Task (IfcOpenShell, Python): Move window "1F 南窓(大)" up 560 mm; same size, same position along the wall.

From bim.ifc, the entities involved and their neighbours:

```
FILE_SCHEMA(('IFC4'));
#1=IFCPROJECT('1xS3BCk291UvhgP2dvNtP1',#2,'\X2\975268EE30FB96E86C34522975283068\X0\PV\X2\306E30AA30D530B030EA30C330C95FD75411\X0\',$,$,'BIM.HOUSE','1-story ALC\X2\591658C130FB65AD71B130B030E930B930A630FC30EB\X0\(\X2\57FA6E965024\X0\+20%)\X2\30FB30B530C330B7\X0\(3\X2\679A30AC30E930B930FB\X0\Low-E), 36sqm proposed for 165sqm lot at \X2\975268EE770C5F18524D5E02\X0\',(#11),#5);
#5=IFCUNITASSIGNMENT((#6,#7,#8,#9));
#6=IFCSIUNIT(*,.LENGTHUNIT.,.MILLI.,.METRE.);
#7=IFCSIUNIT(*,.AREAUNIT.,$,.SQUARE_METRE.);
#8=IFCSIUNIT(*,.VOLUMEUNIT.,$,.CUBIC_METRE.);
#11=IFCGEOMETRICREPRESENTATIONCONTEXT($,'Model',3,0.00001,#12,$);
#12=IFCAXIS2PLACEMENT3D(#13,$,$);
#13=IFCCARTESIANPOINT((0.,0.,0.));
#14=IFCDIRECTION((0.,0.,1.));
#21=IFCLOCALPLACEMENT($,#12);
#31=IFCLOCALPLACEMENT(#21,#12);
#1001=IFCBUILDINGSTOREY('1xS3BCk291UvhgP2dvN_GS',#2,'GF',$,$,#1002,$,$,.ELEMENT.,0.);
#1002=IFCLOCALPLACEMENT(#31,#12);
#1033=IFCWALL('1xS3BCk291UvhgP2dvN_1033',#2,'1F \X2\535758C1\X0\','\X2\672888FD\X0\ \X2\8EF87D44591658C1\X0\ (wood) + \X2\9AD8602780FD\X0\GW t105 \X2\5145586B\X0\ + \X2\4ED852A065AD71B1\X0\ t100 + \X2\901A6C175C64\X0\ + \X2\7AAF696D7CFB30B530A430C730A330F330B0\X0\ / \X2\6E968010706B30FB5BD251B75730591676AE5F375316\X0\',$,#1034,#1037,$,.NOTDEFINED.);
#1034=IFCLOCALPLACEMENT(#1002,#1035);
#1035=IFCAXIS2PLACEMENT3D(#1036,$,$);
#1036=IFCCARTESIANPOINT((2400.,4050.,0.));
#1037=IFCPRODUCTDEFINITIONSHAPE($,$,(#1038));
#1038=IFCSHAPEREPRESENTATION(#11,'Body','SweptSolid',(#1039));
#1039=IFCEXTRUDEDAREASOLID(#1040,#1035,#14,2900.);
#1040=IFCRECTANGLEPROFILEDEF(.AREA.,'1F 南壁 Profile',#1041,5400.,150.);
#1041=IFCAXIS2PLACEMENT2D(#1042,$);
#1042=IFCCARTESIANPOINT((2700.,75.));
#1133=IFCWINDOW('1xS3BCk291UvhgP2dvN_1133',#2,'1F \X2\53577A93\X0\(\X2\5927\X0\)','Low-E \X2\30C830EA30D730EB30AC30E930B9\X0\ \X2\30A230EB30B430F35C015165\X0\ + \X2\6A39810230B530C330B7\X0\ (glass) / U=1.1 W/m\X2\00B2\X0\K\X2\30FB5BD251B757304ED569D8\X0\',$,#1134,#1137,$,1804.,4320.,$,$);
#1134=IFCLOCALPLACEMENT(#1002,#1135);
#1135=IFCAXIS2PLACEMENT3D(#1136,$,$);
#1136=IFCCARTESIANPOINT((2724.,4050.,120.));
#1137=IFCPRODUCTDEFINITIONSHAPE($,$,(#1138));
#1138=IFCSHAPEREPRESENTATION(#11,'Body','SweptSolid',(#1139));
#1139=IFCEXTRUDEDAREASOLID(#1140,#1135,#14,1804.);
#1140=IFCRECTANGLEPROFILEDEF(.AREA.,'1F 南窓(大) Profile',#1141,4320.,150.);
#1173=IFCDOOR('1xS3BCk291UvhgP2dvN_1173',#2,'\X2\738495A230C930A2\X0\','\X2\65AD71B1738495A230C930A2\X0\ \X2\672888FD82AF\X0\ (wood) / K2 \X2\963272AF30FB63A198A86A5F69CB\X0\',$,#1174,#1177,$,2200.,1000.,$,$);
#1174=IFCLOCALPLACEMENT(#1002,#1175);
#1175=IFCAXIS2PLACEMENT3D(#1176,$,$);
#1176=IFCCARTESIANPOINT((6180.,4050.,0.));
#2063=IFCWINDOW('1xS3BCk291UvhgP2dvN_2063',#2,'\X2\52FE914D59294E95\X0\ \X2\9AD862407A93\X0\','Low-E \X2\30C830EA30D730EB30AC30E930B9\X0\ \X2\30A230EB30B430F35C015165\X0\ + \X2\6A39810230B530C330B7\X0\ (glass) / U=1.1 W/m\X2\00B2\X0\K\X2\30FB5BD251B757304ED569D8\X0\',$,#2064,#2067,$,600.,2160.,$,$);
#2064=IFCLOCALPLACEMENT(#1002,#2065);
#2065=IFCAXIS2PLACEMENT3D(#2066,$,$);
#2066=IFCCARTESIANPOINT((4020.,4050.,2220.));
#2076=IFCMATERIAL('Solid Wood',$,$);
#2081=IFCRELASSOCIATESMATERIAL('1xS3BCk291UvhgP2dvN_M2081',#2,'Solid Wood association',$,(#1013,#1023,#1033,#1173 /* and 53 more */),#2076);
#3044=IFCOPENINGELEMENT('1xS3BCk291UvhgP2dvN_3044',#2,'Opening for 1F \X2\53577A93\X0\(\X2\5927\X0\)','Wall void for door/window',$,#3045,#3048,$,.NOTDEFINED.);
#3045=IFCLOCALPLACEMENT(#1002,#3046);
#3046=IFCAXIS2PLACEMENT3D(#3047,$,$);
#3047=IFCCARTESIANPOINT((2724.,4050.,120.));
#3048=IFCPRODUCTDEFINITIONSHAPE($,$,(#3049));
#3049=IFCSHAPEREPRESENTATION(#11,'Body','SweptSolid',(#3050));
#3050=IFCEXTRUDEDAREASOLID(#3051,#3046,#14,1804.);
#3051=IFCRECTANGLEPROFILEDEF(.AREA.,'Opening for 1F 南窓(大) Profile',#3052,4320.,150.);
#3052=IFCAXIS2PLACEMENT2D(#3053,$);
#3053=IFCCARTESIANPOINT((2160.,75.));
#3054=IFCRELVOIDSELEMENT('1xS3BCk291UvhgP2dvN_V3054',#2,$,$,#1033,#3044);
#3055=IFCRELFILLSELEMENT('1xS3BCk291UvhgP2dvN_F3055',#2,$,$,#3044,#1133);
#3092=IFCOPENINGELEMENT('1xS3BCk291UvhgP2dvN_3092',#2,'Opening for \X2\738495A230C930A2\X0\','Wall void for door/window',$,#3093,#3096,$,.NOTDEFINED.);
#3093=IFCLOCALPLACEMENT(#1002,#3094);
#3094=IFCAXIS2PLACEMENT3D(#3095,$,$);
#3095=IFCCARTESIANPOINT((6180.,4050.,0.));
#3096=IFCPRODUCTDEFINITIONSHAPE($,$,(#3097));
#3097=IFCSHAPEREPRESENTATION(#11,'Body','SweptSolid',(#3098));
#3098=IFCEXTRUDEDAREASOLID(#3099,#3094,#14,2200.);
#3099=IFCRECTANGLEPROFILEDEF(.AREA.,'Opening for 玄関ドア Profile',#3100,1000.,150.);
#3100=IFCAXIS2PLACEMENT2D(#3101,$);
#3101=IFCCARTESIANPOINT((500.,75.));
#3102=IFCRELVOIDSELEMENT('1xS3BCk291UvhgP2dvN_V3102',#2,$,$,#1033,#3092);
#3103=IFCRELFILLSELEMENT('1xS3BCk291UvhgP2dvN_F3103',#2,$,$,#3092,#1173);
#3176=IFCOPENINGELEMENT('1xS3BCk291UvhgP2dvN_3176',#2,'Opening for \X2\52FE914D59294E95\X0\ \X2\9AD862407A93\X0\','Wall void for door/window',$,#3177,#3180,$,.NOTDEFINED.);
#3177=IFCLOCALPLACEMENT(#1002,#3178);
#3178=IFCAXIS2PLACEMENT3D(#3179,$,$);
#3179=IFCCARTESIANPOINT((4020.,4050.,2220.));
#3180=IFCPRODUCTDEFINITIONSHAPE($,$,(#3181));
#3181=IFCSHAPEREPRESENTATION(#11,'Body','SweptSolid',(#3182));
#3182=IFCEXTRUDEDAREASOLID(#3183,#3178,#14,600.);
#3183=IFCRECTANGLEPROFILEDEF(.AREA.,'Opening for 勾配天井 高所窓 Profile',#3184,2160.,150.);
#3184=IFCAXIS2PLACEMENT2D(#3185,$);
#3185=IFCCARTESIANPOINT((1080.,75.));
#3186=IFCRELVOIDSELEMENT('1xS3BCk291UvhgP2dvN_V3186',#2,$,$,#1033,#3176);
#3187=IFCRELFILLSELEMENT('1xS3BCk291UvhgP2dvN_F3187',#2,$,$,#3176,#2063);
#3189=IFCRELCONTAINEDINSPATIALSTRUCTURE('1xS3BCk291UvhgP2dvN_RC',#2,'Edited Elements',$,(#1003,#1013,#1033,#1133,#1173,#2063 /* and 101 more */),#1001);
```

```python
import numpy as np
import ifcopenshell
import ifcopenshell.api.geometry
import ifcopenshell.util.placement
import ifcopenshell.util.unit

model = ifcopenshell.open("bim.ifc")
unit_scale = ifcopenshell.util.unit.calculate_unit_scale(model)

window = model.by_id(1133)
opening = window.FillsVoids[0].RelatingOpeningElement
dz = 0.56 / unit_scale

shift = np.array([0.0, 0.0, dz])
# The window is not placed relative to its opening, so move both.
for product in (opening, window):
    matrix = ifcopenshell.util.placement.get_local_placement(product.ObjectPlacement)
    matrix[:3, 3] += shift
    ifcopenshell.api.geometry.edit_object_placement(model, product=product, matrix=matrix, is_si=False)

print(f"moved by {dz * unit_scale:+.3f} m")

model.write("bim-out.ifc")
```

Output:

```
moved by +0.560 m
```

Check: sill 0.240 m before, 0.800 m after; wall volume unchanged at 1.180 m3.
